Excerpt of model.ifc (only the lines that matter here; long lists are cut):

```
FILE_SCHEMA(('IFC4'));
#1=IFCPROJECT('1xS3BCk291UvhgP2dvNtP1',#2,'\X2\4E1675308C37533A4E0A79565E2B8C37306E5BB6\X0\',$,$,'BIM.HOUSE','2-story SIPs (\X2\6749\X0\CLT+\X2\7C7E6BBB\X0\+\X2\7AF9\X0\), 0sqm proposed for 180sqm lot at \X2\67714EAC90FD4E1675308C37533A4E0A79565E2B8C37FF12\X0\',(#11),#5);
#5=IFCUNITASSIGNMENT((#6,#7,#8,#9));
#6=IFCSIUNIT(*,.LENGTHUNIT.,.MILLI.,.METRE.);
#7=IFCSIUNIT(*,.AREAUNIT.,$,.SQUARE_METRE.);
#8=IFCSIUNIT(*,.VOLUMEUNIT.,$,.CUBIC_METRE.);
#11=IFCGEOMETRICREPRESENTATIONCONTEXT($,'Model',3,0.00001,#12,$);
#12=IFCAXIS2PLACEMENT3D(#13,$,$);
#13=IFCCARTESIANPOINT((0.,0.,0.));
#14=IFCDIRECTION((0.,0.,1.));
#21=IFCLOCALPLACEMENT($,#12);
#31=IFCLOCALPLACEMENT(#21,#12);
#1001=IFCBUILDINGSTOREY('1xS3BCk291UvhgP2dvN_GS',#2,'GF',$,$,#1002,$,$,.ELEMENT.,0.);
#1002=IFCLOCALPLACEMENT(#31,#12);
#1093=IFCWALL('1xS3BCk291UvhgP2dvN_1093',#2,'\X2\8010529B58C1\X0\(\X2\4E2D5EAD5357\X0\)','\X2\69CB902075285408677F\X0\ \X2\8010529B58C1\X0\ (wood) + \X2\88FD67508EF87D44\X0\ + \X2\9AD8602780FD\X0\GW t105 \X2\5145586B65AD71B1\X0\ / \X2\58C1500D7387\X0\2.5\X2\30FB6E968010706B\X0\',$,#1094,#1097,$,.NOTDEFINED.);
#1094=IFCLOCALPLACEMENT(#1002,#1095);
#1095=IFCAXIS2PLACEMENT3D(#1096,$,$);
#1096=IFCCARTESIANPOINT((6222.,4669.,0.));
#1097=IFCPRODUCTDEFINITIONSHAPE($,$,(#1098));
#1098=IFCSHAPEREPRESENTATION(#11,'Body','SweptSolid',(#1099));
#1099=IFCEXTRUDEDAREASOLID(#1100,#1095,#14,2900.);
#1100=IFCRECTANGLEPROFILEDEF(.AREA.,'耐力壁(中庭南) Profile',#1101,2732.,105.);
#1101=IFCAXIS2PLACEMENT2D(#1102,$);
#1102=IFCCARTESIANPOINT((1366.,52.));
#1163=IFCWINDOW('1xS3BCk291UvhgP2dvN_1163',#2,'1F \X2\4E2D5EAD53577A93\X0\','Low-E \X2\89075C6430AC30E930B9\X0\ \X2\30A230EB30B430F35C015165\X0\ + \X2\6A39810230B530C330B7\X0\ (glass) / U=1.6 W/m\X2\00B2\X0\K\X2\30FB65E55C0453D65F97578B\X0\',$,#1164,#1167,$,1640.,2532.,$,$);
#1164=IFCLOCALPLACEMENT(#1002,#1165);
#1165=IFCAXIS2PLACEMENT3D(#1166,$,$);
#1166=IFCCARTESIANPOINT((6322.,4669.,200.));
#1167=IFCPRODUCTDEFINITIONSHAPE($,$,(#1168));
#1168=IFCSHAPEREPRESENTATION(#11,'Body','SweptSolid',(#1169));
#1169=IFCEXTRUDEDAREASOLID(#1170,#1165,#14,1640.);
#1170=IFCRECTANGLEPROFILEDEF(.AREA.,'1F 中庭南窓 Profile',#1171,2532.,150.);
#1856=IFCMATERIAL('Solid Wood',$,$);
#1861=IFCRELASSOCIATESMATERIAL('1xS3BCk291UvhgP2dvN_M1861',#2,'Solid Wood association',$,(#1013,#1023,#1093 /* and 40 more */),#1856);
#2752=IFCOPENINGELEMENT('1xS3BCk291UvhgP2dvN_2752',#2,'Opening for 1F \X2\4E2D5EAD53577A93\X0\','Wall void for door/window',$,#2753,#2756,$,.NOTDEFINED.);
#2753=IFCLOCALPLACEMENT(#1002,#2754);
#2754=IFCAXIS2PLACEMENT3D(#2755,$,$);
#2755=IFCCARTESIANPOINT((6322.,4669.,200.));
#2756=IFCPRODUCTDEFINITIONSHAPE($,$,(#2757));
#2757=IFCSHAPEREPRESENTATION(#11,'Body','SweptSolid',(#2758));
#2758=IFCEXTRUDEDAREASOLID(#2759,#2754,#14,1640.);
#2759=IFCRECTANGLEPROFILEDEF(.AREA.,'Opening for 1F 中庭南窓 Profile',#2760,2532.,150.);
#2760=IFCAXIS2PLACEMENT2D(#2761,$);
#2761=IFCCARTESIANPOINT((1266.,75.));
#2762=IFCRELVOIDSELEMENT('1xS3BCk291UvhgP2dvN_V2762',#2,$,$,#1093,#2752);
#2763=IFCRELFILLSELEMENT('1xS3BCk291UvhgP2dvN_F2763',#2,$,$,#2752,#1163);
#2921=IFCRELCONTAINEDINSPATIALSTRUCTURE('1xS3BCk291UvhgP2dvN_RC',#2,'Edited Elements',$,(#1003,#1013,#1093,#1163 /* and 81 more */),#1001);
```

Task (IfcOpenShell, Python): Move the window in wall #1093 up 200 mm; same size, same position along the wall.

```python
import numpy as np
import ifcopenshell
import ifcopenshell.api.geometry
import ifcopenshell.util.placement
import ifcopenshell.util.unit

model = ifcopenshell.open("model.ifc")
unit_scale = ifcopenshell.util.unit.calculate_unit_scale(model)

window = model.by_guid("1xS3BCk291UvhgP2dvN_1163")
opening = window.FillsVoids[0].RelatingOpeningElement
dz = 0.2 / unit_scale

shift = np.array([0.0, 0.0, dz])
# The window is not placed relative to its opening, so move both.
for product in (opening, window):
    matrix = ifcopenshell.util.placement.get_local_placement(product.ObjectPlacement)
    matrix[:3, 3] += shift
    ifcopenshell.api.geometry.edit_object_placement(model, product=product, matrix=matrix, is_si=False)

print(f"moved by {dz * unit_scale:+.3f} m")

model.write("model_rev.ifc")
```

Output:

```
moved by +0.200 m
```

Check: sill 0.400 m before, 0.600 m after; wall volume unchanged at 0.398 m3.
